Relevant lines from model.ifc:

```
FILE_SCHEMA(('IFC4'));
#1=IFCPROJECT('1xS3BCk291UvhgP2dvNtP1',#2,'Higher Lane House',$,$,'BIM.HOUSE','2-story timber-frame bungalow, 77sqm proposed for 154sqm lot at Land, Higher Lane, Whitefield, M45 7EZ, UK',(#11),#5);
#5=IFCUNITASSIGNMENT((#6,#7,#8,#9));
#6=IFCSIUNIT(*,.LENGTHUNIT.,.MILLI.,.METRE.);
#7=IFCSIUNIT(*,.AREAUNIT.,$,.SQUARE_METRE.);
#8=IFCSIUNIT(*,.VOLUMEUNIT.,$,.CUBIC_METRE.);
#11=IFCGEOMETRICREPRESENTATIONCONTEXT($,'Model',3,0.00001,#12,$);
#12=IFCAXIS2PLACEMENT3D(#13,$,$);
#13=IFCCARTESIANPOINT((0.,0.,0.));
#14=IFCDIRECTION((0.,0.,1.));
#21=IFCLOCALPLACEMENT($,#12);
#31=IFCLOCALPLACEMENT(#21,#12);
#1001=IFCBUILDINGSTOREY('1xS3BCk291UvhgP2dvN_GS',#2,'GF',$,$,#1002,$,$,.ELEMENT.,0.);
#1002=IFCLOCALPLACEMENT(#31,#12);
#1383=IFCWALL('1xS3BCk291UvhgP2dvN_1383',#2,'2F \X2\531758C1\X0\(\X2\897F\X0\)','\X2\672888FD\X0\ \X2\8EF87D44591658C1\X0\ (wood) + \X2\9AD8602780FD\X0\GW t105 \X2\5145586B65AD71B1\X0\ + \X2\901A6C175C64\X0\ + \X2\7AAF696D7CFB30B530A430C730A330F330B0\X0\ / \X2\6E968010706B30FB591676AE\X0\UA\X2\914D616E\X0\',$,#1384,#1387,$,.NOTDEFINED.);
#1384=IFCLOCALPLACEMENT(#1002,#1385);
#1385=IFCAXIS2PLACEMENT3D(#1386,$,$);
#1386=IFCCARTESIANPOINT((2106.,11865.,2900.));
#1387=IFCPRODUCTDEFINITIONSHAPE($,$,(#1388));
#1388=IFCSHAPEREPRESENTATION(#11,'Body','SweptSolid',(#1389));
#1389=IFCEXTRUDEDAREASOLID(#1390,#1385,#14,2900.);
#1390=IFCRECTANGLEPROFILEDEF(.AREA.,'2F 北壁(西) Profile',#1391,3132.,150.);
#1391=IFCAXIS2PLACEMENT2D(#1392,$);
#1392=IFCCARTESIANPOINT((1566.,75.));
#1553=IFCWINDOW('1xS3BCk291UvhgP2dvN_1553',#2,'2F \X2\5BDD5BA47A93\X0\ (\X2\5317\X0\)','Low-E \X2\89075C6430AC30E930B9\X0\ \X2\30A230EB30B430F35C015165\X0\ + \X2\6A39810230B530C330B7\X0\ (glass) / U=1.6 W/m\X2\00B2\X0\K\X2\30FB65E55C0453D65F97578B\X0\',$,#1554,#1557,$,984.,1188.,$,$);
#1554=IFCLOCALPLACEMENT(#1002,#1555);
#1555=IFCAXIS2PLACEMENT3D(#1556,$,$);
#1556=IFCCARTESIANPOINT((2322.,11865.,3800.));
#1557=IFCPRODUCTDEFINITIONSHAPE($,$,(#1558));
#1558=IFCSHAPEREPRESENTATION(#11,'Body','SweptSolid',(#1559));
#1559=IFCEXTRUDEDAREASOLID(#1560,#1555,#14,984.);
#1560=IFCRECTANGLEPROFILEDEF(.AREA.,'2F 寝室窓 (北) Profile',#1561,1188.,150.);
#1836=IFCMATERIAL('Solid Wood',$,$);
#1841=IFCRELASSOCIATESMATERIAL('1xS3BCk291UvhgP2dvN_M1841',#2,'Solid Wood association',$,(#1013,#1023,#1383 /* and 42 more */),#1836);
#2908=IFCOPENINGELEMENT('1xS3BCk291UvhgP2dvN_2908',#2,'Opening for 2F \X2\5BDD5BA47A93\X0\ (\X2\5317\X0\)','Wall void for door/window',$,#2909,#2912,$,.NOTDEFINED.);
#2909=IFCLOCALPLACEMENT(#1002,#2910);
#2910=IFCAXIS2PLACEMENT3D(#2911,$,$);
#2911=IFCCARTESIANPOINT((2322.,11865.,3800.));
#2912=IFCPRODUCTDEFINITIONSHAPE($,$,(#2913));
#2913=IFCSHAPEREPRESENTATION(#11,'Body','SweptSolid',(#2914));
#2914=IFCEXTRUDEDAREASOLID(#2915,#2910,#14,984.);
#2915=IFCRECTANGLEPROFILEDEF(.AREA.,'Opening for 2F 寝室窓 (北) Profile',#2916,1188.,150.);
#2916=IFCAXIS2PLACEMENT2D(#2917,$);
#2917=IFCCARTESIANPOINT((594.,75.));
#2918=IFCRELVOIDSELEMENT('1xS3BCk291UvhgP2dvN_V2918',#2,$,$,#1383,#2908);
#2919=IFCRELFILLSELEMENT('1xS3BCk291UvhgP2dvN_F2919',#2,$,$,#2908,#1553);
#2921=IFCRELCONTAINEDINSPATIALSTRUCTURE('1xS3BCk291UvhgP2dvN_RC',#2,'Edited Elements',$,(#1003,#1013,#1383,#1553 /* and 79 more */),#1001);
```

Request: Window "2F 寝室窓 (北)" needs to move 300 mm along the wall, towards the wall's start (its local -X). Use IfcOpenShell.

```python
import ifcopenshell
import ifcopenshell.api.geometry
import ifcopenshell.util.placement
import ifcopenshell.util.unit

model = ifcopenshell.open("model.ifc")
unit_scale = ifcopenshell.util.unit.calculate_unit_scale(model)

window = model.by_id(1553)
opening = window.FillsVoids[0].RelatingOpeningElement
wall = opening.VoidsElements[0].RelatingBuildingElement

wall_matrix = ifcopenshell.util.placement.get_local_placement(wall.ObjectPlacement)
shift = wall_matrix[:3, 0] * -0.3 / unit_scale
before = ifcopenshell.util.placement.get_local_placement(window.ObjectPlacement)[:3, 3].copy()

# The window is not placed relative to its opening, so move both.
for product in (opening, window):
    matrix = ifcopenshell.util.placement.get_local_placement(product.ObjectPlacement)
    matrix[:3, 3] += shift
    ifcopenshell.api.geometry.edit_object_placement(model, product=product, matrix=matrix, is_si=False)

after = ifcopenshell.util.placement.get_local_placement(window.ObjectPlacement)[:3, 3]
print("window moved by", (after - before).round(3) + 0.0)

model.write("model-out.ifc")
```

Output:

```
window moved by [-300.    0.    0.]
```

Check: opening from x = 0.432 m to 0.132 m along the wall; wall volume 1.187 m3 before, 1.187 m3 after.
